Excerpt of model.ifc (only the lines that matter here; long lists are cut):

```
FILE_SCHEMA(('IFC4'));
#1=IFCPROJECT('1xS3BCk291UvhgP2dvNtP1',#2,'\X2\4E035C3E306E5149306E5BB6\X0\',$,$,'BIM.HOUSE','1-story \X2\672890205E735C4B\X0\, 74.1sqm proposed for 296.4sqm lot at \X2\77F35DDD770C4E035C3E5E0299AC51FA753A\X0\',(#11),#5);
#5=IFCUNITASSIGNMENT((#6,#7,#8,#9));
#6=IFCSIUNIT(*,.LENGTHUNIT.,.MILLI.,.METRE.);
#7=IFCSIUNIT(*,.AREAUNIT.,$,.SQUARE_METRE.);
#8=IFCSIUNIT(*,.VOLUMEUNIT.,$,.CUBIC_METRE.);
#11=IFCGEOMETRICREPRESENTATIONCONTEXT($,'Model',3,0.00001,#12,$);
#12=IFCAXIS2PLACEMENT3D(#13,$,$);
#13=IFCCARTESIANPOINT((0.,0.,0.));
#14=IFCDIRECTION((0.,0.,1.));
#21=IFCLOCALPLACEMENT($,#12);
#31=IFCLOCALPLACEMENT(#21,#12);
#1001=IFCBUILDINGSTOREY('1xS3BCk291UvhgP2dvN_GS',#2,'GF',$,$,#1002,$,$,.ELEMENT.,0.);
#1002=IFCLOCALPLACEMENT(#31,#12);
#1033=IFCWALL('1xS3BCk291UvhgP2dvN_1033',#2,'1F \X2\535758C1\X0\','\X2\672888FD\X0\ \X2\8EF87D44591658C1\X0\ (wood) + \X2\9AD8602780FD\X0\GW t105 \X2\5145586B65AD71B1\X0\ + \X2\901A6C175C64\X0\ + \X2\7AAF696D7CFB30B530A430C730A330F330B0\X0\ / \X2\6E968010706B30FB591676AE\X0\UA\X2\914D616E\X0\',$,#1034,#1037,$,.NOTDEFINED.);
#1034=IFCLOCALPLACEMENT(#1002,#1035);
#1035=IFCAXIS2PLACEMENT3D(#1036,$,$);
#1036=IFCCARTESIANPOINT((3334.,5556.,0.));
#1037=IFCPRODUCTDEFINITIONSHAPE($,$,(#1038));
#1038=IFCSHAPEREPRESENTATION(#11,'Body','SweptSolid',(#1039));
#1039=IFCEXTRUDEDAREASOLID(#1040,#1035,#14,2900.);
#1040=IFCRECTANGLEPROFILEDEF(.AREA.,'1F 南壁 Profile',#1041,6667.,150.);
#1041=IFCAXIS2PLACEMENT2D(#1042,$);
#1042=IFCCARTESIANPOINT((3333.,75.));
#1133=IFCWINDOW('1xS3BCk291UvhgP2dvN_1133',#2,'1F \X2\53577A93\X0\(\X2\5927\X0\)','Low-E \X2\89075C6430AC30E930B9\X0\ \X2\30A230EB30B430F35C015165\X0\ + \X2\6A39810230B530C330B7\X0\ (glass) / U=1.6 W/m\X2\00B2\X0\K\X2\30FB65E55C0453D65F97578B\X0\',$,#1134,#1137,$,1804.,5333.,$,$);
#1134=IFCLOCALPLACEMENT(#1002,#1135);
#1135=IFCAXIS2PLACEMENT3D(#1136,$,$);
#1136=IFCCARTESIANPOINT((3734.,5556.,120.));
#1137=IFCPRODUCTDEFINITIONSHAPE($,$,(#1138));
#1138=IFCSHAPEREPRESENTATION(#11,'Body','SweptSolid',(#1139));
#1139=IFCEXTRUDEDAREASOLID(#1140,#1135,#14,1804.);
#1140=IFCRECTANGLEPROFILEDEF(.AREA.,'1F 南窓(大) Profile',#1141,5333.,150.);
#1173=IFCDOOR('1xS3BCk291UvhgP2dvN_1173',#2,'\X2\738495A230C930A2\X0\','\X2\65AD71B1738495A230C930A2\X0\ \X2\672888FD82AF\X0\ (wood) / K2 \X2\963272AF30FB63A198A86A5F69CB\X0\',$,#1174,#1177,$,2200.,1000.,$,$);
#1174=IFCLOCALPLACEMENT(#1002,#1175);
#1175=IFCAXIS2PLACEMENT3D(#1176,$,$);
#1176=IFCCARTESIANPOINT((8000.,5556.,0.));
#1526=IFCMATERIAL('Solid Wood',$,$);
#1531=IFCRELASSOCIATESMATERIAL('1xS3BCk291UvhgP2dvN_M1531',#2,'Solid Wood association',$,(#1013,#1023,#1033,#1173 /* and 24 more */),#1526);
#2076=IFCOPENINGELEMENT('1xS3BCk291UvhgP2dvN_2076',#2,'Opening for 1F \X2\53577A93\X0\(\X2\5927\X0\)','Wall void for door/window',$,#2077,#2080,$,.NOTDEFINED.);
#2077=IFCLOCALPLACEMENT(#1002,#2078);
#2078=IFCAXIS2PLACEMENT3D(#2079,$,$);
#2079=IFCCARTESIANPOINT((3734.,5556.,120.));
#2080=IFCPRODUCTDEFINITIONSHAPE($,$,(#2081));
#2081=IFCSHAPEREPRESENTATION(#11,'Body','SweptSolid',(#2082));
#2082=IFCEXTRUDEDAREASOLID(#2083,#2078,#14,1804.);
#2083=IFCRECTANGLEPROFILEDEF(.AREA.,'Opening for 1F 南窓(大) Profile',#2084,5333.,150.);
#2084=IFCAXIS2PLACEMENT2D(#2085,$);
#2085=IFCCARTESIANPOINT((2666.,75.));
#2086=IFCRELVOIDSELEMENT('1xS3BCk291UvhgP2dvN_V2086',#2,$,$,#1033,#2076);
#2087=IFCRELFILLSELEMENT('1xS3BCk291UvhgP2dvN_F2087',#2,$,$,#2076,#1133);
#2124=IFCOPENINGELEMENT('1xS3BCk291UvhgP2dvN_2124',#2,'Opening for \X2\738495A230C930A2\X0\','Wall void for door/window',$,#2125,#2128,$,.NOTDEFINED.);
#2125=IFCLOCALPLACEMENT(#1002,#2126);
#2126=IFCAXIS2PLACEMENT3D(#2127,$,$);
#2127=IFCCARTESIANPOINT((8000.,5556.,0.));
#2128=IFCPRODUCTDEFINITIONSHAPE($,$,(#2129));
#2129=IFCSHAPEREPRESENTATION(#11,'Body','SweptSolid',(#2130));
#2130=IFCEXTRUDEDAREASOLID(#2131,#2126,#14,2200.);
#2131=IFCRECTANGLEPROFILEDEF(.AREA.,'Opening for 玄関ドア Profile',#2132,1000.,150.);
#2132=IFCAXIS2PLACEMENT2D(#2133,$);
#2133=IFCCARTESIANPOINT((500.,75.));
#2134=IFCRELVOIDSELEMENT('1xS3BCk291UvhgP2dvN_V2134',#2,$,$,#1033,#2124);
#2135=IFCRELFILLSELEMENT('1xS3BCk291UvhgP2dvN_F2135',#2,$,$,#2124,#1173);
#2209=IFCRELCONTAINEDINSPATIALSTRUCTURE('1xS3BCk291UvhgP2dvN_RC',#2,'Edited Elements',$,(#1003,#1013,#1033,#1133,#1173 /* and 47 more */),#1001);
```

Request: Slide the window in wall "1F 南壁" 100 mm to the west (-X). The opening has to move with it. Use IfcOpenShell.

```python
import ifcopenshell
import ifcopenshell.api.geometry
import ifcopenshell.util.placement
import ifcopenshell.util.unit

model = ifcopenshell.open("model.ifc")
unit_scale = ifcopenshell.util.unit.calculate_unit_scale(model)

window = model.by_id(1133)
opening = window.FillsVoids[0].RelatingOpeningElement
wall = opening.VoidsElements[0].RelatingBuildingElement

wall_matrix = ifcopenshell.util.placement.get_local_placement(wall.ObjectPlacement)
shift = wall_matrix[:3, 0] * -0.1 / unit_scale
before = ifcopenshell.util.placement.get_local_placement(window.ObjectPlacement)[:3, 3].copy()

# The window is not placed relative to its opening, so move both.
for product in (opening, window):
    matrix = ifcopenshell.util.placement.get_local_placement(product.ObjectPlacement)
    matrix[:3, 3] += shift
    ifcopenshell.api.geometry.edit_object_placement(model, product=product, matrix=matrix, is_si=False)

after = ifcopenshell.util.placement.get_local_placement(window.ObjectPlacement)[:3, 3]
print("window moved by", (after - before).round(3) + 0.0)

model.write("model_updated.ifc")
```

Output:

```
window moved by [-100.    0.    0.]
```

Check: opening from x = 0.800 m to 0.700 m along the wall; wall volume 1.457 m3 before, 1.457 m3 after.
